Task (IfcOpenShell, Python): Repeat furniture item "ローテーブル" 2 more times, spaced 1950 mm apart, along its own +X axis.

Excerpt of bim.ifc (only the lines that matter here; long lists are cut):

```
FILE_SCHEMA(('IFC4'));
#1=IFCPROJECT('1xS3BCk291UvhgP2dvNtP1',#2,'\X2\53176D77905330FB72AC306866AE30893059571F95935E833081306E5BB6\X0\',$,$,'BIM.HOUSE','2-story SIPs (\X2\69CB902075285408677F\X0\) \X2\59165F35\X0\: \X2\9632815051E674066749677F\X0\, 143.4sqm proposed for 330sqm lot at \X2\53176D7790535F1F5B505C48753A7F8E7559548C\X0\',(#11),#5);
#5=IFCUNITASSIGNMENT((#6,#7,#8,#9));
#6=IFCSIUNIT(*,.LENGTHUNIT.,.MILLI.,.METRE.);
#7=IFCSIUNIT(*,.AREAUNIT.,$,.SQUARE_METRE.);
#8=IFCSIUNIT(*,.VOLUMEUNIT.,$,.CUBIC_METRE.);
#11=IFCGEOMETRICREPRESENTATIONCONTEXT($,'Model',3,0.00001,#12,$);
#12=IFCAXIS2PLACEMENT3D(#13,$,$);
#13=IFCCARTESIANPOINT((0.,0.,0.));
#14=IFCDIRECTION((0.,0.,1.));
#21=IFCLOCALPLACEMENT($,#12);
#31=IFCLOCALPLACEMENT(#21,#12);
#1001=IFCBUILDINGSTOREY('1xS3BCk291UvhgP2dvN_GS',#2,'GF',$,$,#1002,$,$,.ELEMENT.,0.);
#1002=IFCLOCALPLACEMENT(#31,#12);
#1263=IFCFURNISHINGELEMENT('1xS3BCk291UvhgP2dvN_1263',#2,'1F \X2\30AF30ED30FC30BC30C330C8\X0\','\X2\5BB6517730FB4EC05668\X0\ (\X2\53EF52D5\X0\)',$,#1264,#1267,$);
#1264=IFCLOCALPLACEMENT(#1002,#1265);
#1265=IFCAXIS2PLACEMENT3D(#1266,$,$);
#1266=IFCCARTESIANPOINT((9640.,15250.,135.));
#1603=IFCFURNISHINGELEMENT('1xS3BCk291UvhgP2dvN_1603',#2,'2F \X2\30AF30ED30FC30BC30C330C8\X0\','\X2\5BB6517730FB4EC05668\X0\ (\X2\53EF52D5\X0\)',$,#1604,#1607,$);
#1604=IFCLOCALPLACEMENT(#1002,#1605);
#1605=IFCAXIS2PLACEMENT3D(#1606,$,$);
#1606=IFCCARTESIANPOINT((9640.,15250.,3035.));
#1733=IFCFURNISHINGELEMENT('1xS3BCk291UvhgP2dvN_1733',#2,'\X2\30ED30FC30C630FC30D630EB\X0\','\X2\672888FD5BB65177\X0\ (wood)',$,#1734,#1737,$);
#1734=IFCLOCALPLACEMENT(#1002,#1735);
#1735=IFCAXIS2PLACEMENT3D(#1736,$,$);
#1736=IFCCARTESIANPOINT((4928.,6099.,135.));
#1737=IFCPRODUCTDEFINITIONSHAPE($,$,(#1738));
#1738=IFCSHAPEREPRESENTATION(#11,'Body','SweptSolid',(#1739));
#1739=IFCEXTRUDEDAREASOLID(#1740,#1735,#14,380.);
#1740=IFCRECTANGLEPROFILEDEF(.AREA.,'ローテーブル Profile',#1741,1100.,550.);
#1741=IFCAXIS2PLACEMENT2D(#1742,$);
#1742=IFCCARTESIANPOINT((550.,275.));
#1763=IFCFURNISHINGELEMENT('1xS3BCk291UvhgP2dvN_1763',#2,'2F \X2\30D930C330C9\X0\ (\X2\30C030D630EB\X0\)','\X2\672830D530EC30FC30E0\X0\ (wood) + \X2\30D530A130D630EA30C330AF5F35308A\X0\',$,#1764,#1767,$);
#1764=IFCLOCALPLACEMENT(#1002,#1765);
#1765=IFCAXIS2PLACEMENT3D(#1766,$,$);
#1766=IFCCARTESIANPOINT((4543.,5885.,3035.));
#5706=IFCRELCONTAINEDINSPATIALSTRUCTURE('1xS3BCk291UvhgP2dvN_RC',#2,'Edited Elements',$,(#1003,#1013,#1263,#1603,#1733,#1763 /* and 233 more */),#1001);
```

```python
import ifcopenshell
import ifcopenshell.api.geometry
import ifcopenshell.api.root
import ifcopenshell.util.element
import ifcopenshell.util.placement
import ifcopenshell.util.unit

model = ifcopenshell.open("bim.ifc")
unit_scale = ifcopenshell.util.unit.calculate_unit_scale(model)


def reuse_history(source, copy):
    """copy_class also copies each property set's owner history, people and application; keep the originals."""
    for rel in copy.IsDefinedBy:
        if rel.is_a("IfcRelDefinesByProperties") and (history := rel.RelatingPropertyDefinition.OwnerHistory):
            rel.RelatingPropertyDefinition.OwnerHistory = source.OwnerHistory
            ifcopenshell.util.element.remove_deep2(model, history)


source = model.by_id(1733)
base = ifcopenshell.util.placement.get_local_placement(source.ObjectPlacement)
step = base[:3, 0] * 1.95 / unit_scale

for i in range(1, 3):
    copy = ifcopenshell.api.root.copy_class(model, product=source)
    copy.Representation = ifcopenshell.util.element.copy_deep(
        model, source.Representation, exclude=["IfcGeometricRepresentationContext", "IfcRepresentationMap"]
    )
    reuse_history(source, copy)
    matrix = base.copy()
    matrix[:3, 3] += i * step
    print("added at", matrix[:3, 3].round(3) + 0.0)
    ifcopenshell.api.geometry.edit_object_placement(model, product=copy, matrix=matrix, is_si=False)

model.write("bim_edited.ifc")
```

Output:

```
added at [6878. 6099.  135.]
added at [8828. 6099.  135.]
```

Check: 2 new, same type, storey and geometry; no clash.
